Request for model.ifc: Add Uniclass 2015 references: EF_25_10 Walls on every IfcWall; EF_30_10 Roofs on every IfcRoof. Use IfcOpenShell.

First a look at what the model holds.

```python
import ifcopenshell

model = ifcopenshell.open("model.ifc")
print(model.schema)
print("classifications:", [c.Name for c in model.by_type("IfcClassification")])
for ifc_class in ("IfcDoor", "IfcRoof", "IfcStair", "IfcWall", "IfcWindow"):
    print(ifc_class, len(model.by_type(ifc_class)))
```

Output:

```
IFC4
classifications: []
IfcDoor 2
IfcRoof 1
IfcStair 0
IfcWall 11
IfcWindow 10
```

```python
import ifcopenshell
import ifcopenshell.api.classification

model = ifcopenshell.open("model.ifc")

system = ifcopenshell.api.classification.add_classification(model, classification="Uniclass 2015")

codes = {
    "IfcWall": ("EF_25_10", "Walls"),
    "IfcRoof": ("EF_30_10", "Roofs"),
}
for ifc_class, (code, name) in codes.items():
    products = model.by_type(ifc_class)
    ifcopenshell.api.classification.add_reference(
        model, products=products, classification=system, identification=code, name=name
    )
    print(code, len(products))

model.write("model_edited.ifc")
```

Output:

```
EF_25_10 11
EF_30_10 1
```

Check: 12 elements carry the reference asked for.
